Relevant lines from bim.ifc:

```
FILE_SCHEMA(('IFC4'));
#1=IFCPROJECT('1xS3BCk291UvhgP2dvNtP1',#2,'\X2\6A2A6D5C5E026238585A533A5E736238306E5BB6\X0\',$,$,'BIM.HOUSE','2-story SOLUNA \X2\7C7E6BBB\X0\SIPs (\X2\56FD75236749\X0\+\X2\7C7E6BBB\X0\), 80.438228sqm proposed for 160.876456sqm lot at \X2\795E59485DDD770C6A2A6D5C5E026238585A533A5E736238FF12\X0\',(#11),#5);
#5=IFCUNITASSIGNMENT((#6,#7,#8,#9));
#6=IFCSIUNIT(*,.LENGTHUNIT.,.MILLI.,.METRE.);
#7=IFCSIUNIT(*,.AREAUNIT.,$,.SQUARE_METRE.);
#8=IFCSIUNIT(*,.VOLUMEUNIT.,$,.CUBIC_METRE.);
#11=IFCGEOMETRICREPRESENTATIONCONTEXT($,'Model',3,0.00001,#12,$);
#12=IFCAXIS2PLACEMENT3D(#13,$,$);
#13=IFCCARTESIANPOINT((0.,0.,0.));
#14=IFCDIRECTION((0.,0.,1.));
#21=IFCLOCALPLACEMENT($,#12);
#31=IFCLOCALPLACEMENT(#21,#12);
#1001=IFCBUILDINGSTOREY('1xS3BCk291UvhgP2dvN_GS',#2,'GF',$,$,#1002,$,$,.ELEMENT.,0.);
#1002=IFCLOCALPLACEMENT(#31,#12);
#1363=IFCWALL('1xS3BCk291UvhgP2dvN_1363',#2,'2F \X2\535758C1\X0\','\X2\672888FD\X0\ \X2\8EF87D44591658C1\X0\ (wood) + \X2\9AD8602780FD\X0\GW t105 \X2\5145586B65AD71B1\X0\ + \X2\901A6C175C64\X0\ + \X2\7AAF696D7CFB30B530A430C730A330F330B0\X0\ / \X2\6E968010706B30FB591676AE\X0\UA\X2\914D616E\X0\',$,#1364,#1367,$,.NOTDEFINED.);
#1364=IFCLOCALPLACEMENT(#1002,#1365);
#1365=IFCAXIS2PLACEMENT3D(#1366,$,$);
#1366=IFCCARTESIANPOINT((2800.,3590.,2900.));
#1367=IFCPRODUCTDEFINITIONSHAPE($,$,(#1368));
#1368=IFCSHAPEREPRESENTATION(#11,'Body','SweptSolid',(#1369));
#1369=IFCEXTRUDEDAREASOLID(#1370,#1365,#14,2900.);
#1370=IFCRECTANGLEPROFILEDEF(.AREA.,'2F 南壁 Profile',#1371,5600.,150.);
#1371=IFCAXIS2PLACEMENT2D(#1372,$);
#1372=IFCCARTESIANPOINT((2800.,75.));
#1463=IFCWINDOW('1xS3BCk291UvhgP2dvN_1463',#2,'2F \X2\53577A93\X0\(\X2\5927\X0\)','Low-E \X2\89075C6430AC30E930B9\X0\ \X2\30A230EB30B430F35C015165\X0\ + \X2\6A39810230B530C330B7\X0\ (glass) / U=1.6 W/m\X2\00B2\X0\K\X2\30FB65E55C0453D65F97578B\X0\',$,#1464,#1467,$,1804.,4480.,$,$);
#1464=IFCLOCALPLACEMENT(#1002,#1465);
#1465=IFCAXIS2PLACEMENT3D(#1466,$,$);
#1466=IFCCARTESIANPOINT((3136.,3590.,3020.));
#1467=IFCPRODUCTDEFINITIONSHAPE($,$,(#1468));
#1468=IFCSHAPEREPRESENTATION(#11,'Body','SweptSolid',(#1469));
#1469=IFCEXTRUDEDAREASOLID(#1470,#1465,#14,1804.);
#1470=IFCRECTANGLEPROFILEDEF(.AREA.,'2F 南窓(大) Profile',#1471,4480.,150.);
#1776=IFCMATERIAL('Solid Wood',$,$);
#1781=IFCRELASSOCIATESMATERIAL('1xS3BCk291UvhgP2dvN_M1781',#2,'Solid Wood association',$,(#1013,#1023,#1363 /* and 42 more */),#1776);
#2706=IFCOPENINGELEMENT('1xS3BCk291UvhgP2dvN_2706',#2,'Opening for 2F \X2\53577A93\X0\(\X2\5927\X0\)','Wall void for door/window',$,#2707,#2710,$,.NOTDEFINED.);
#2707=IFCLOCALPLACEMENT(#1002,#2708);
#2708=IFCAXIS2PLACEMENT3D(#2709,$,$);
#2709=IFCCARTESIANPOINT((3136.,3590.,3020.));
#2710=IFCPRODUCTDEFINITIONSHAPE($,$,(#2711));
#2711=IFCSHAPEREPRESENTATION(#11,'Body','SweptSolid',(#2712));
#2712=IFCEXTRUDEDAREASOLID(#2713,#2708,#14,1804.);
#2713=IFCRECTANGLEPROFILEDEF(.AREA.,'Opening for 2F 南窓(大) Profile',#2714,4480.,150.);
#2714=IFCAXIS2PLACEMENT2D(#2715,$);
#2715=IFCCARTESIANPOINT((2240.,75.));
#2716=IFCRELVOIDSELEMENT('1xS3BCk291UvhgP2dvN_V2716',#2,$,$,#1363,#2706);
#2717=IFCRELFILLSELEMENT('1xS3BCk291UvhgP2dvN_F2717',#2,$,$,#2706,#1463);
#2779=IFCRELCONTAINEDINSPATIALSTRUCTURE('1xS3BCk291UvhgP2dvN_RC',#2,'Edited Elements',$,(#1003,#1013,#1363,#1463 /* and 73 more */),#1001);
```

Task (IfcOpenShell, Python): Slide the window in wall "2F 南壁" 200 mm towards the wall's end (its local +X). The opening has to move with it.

```python
import ifcopenshell
import ifcopenshell.api.geometry
import ifcopenshell.util.placement

model = ifcopenshell.open("bim.ifc")

window = model.by_guid("1xS3BCk291UvhgP2dvN_1463")
opening = window.FillsVoids[0].RelatingOpeningElement
wall = opening.VoidsElements[0].RelatingBuildingElement

wall_matrix = ifcopenshell.util.placement.get_local_placement(wall.ObjectPlacement)
shift = wall_matrix[:3, 0] * 200.0
before = ifcopenshell.util.placement.get_local_placement(window.ObjectPlacement)[:3, 3].copy()

# The window is not placed relative to its opening, so move both.
for product in (opening, window):
    matrix = ifcopenshell.util.placement.get_local_placement(product.ObjectPlacement)
    matrix[:3, 3] += shift
    ifcopenshell.api.geometry.edit_object_placement(model, product=product, matrix=matrix, is_si=False)

after = ifcopenshell.util.placement.get_local_placement(window.ObjectPlacement)[:3, 3]
print("window moved by", (after - before).round(3) + 0.0)

model.write("bim_updated.ifc")
```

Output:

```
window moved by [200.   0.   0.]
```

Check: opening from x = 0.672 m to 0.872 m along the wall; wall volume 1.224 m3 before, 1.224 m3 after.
